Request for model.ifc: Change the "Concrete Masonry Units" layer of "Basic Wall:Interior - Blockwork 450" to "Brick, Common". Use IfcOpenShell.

First a look at what the model holds.

```python
import ifcopenshell
import ifcopenshell.util.element

model = ifcopenshell.open("model.ifc")
print(model.schema)
for layer_set in model.by_type("IfcMaterialLayerSet"):
    if layer_set.LayerSetName == "Basic Wall:Interior - Blockwork 450":
        for layer in layer_set.MaterialLayers:
            print(layer.id(), layer.Material and layer.Material.Name, layer.LayerThickness, sep=" | ")
        print(len(ifcopenshell.util.element.get_elements_by_material(model, layer_set)), "elements and types use it")
print(sorted(m.Name for m in model.by_type("IfcMaterial") if m.Name)[:60])
```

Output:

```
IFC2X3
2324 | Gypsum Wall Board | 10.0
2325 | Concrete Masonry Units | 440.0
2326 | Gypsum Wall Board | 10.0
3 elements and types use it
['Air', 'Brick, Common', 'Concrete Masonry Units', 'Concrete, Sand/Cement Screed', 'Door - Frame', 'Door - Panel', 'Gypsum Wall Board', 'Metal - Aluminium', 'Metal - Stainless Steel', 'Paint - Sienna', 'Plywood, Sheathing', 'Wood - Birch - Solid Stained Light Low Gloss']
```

```python
import ifcopenshell
import ifcopenshell.api.material

model = ifcopenshell.open("model.ifc")

layer_set = next(s for s in model.by_type("IfcMaterialLayerSet") if s.LayerSetName == "Basic Wall:Interior - Blockwork 450")
layer = next(l for l in layer_set.MaterialLayers if l.Material and l.Material.Name == "Concrete Masonry Units")
material = next(m for m in model.by_type("IfcMaterial") if m.Name == "Brick, Common")

# Point this one layer at the other material; renaming the old one would change it everywhere.
ifcopenshell.api.material.edit_layer(model, layer=layer, attributes={}, material=material)

print([l.Material.Name if l.Material else None for l in layer_set.MaterialLayers])

model.write("model_rev.ifc")
```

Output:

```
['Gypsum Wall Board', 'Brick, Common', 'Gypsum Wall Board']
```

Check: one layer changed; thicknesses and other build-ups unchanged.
